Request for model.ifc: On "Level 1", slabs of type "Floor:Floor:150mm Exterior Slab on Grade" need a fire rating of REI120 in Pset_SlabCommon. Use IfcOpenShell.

First a look at what the model holds.

```python
import ifcopenshell
import ifcopenshell.util.element

model = ifcopenshell.open("model.ifc")
print(model.schema)
storey = next(s for s in model.by_type("IfcBuildingStorey") if s.Name == "Level 1")
slabs = [e for e in ifcopenshell.util.element.get_decomposition(storey) if e.is_a("IfcSlab")]
seen = {}
for e in slabs:
    element_type = ifcopenshell.util.element.get_type(e)
    key = (element_type.Name if element_type != e and element_type else None, ifcopenshell.util.element.get_pset(e, "Pset_SlabCommon", "FireRating"))
    seen[key] = seen.get(key, 0) + 1
for (name, value), count in sorted(seen.items(), key=str):
    print(count, "x", name, "|", value)
```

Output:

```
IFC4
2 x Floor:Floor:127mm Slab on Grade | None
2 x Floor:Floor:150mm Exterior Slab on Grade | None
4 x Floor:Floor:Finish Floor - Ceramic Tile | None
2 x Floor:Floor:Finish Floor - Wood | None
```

```python
import ifcopenshell
import ifcopenshell.api.pset
import ifcopenshell.util.element

model = ifcopenshell.open("model.ifc")

storey = next(s for s in model.by_type("IfcBuildingStorey") if s.Name == "Level 1")
slabs = [e for e in ifcopenshell.util.element.get_decomposition(storey) if e.is_a("IfcSlab")]

count = 0
for e in slabs:
    element_type = ifcopenshell.util.element.get_type(e)
    if element_type in (None, e) or element_type.Name != "Floor:Floor:150mm Exterior Slab on Grade":
        continue
    # add_pset returns the element's existing set when there is one.
    pset = ifcopenshell.api.pset.add_pset(model, product=e, name="Pset_SlabCommon")
    ifcopenshell.api.pset.edit_pset(model, pset=pset, properties={"FireRating": "REI120"})
    count += 1

print(count, "slabs updated")

model.write("model_v2.ifc")
```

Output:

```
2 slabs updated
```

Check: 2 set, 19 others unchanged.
